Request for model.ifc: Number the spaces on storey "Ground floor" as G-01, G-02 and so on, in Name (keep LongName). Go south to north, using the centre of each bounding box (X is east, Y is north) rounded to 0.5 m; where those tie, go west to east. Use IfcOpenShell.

First a look at what the model holds.

```python
import ifcopenshell
import ifcopenshell.util.element
import ifcopenshell.util.placement

model = ifcopenshell.open("model.ifc")
print(model.schema)
storey = next(s for s in model.by_type("IfcBuildingStorey") if s.Name == "Ground floor")
spaces = [e for e in ifcopenshell.util.element.get_decomposition(storey) if e.is_a("IfcSpace")]
for e in sorted(spaces, key=lambda e: e.id()):
    origin = ifcopenshell.util.placement.get_local_placement(e.ObjectPlacement)[:3, 3]
    print(e.id(), e.Name, e.LongName, origin.round(2) + 0.0, sep=" | ")
```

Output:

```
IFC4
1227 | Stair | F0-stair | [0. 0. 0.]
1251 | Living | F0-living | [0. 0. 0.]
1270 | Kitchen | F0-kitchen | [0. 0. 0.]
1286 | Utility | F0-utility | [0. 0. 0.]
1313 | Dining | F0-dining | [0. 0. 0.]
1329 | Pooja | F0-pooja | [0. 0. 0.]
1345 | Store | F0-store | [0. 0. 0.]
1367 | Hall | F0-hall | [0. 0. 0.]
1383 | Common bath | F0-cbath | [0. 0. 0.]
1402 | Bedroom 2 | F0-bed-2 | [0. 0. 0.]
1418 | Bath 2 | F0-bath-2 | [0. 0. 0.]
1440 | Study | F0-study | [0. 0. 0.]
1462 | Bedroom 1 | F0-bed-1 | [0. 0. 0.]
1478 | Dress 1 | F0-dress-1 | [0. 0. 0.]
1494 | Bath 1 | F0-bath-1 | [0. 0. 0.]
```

```python
import ifcopenshell
import ifcopenshell.geom
import ifcopenshell.util.element
import ifcopenshell.util.shape

model = ifcopenshell.open("model.ifc")
settings = ifcopenshell.geom.settings()
settings.set("use-world-coords", True)


def centre(element):
    shape = ifcopenshell.geom.create_shape(settings, element)
    return ifcopenshell.util.shape.get_bbox_centroid(shape.geometry)


storey = next(s for s in model.by_type("IfcBuildingStorey") if s.Name == "Ground floor")
spaces = [e for e in ifcopenshell.util.element.get_decomposition(storey) if e.is_a("IfcSpace")]

# Insertion points can sit at a corner or the storey origin, so sort by the geometry (in metres).
centres = {e: centre(e) for e in spaces}
spaces.sort(key=lambda e: (round(centres[e][1] / 0.5), centres[e][0]))

for i, e in enumerate(spaces, start=1):
    number = f"G-{i:02d}"
    e.Name = number
    print(e.id(), number)

model.write("model_updated.ifc")
```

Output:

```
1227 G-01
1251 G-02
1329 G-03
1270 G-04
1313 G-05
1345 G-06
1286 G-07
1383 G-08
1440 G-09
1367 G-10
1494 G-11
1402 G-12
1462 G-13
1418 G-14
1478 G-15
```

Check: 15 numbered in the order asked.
